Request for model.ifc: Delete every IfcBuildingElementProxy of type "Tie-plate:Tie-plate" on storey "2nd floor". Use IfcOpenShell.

First a look at what the model holds.

```python
import ifcopenshell
import ifcopenshell.util.element

model = ifcopenshell.open("model.ifc")
print(model.schema)
storey = next(s for s in model.by_type("IfcBuildingStorey") if s.Name == "2nd floor")
proxies = [e for e in ifcopenshell.util.element.get_decomposition(storey) if e.is_a("IfcBuildingElementProxy")]
seen = {}
for e in proxies:
    element_type = ifcopenshell.util.element.get_type(e)
    name = element_type.Name if element_type not in (None, e) else None
    seen[name] = seen.get(name, 0) + 1
for name, count in sorted(seen.items(), key=str):
    print(count, "x", name)
```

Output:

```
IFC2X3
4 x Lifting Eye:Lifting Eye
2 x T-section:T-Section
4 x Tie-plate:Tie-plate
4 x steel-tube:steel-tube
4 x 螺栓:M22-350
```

```python
import ifcopenshell
import ifcopenshell.api.root
import ifcopenshell.util.element

model = ifcopenshell.open("model.ifc")

storey = next(s for s in model.by_type("IfcBuildingStorey") if s.Name == "2nd floor")
proxies = [e for e in ifcopenshell.util.element.get_decomposition(storey) if e.is_a("IfcBuildingElementProxy")]
targets = [e for e in proxies if (t := ifcopenshell.util.element.get_type(e)) not in (None, e) and t.Name == "Tie-plate:Tie-plate"]

for e in targets:
    ifcopenshell.api.root.remove_product(model, product=e)
print(len(targets), "removed")

model.write("model_rev.ifc")
```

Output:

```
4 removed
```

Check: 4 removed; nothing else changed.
